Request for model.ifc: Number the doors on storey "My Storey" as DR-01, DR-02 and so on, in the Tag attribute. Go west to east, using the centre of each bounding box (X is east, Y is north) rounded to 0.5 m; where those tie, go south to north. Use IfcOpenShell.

First a look at what the model holds.

```python
import ifcopenshell
import ifcopenshell.util.element
import ifcopenshell.util.placement

model = ifcopenshell.open("model.ifc")
print(model.schema)
storey = next(s for s in model.by_type("IfcBuildingStorey") if s.Name == "My Storey")
doors = [e for e in ifcopenshell.util.element.get_decomposition(storey) if e.is_a("IfcDoor")]
for e in sorted(doors, key=lambda e: e.id()):
    origin = ifcopenshell.util.placement.get_local_placement(e.ObjectPlacement)[:3, 3]
    print(e.id(), e.Tag, e.Name, origin.round(2) + 0.0, sep=" | ")
```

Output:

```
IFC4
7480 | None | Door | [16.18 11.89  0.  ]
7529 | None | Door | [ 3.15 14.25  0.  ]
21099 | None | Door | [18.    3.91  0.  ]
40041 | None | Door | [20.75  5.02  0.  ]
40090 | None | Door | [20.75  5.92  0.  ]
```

```python
import ifcopenshell
import ifcopenshell.geom
import ifcopenshell.util.element
import ifcopenshell.util.shape

model = ifcopenshell.open("model.ifc")
settings = ifcopenshell.geom.settings()
settings.set("use-world-coords", True)


def centre(element):
    shape = ifcopenshell.geom.create_shape(settings, element)
    return ifcopenshell.util.shape.get_bbox_centroid(shape.geometry)


storey = next(s for s in model.by_type("IfcBuildingStorey") if s.Name == "My Storey")
doors = [e for e in ifcopenshell.util.element.get_decomposition(storey) if e.is_a("IfcDoor")]

# Insertion points can sit at a corner or the storey origin, so sort by the geometry (in metres).
centres = {e: centre(e) for e in doors}
doors.sort(key=lambda e: (round(centres[e][0] / 0.5), centres[e][1]))

for i, e in enumerate(doors, start=1):
    number = f"DR-{i:02d}"
    e.Tag = number
    print(e.id(), number)

model.write("model_rev.ifc")
```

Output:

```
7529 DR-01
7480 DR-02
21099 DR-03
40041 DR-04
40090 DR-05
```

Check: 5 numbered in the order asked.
